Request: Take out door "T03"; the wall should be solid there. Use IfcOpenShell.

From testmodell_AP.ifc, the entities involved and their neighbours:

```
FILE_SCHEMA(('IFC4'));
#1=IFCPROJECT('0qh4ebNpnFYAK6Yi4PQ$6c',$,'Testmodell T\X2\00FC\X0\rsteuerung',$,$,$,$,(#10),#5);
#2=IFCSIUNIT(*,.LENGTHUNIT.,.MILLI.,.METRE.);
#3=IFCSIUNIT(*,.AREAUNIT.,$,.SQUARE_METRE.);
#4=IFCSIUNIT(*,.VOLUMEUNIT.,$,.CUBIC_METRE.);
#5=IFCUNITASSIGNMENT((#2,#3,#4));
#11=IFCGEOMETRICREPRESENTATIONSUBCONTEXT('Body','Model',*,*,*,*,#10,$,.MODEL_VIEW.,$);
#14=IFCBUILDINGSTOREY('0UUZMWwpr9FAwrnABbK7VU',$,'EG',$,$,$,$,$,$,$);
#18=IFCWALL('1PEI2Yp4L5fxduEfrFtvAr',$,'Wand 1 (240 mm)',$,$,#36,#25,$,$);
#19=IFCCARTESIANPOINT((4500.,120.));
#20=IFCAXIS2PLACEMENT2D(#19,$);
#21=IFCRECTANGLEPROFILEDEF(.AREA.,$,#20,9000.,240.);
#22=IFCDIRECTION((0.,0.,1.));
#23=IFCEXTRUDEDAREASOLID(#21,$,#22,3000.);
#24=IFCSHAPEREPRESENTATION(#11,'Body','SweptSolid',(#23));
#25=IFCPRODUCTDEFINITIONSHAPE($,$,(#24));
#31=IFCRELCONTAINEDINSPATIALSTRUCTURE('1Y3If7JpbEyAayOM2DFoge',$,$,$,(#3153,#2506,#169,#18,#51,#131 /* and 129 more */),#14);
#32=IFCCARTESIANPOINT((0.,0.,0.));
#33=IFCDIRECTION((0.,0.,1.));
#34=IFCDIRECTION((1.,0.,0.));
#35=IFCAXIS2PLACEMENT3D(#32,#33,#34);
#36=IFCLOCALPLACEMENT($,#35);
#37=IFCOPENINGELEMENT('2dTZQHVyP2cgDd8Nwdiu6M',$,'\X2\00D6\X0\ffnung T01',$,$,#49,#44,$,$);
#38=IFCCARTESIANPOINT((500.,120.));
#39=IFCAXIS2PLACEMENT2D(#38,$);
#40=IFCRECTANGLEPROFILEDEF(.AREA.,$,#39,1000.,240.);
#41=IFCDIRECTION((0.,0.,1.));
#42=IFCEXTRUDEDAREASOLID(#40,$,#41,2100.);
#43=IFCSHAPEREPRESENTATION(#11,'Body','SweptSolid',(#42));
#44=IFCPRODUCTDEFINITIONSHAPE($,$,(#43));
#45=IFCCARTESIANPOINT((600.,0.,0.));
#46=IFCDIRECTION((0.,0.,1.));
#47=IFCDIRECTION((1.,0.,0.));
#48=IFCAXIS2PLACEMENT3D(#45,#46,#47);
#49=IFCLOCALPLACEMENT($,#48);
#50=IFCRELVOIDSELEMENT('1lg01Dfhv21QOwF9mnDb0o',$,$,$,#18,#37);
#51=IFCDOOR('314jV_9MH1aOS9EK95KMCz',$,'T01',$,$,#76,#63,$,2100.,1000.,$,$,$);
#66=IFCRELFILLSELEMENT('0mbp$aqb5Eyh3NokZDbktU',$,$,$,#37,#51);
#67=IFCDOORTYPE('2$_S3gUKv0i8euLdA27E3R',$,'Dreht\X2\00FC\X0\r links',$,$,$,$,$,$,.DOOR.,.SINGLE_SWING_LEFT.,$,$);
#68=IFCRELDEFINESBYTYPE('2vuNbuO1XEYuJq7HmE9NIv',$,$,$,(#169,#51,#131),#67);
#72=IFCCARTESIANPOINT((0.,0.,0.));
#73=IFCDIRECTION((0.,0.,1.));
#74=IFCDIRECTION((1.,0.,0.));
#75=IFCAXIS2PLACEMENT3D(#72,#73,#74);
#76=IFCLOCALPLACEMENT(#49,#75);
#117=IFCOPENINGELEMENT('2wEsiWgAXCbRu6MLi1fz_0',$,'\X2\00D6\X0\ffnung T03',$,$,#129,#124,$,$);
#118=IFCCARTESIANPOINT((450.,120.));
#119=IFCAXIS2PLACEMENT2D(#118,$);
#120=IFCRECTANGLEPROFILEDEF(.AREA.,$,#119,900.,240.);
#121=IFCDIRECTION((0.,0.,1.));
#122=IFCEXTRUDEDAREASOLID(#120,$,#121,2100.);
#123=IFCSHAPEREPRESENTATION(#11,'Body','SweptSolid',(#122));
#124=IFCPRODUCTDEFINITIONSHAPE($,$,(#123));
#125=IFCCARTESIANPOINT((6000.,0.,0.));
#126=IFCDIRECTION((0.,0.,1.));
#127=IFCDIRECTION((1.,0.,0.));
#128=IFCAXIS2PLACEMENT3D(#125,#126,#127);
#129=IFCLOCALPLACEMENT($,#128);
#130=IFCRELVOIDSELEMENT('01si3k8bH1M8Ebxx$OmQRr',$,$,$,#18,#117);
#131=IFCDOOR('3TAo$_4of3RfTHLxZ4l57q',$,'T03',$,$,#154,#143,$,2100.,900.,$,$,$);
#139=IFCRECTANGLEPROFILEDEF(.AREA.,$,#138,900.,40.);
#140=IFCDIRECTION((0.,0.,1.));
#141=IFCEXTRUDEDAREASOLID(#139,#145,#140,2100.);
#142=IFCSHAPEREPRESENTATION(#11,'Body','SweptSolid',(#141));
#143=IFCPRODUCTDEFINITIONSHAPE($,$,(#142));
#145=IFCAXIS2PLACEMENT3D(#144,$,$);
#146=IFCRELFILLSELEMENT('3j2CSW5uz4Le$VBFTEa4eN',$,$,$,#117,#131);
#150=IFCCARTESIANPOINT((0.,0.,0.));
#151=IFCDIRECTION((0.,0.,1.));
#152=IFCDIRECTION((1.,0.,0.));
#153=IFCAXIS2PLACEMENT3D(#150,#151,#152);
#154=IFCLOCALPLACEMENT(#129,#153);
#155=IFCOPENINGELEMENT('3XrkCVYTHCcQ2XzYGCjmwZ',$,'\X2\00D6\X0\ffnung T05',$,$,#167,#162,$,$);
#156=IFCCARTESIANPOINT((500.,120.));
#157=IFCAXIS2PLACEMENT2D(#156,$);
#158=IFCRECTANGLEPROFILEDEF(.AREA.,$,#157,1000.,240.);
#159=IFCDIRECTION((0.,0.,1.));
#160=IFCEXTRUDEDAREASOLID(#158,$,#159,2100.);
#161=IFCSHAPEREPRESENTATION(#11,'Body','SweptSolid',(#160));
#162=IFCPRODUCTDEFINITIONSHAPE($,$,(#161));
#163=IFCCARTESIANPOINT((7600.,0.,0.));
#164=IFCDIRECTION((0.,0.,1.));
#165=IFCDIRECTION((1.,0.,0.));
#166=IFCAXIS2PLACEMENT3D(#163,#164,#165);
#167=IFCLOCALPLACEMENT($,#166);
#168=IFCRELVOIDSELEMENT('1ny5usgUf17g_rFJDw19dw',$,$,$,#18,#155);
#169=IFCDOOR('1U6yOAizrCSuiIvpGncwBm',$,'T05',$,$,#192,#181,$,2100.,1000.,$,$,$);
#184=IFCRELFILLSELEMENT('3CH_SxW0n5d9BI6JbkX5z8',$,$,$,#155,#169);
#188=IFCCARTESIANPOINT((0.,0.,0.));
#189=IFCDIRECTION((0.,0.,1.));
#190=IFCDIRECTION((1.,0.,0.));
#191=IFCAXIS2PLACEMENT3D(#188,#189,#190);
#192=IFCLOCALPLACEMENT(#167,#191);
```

```python
import ifcopenshell
import ifcopenshell.api.feature
import ifcopenshell.api.root
import ifcopenshell.geom
import ifcopenshell.util.shape

model = ifcopenshell.open("testmodell_AP.ifc")
settings = ifcopenshell.geom.settings()


def volume(element):
    """Net volume in cubic metres, openings subtracted."""
    shape = ifcopenshell.geom.create_shape(settings, element)
    return ifcopenshell.util.shape.get_volume(shape.geometry)


door = model.by_guid("3TAo$_4of3RfTHLxZ4l57q")
opening = door.FillsVoids[0].RelatingOpeningElement
wall = opening.VoidsElements[0].RelatingBuildingElement
before = volume(wall)

ifcopenshell.api.root.remove_product(model, product=door)
ifcopenshell.api.feature.remove_feature(model, feature=opening)

after = volume(wall)

print(f"wall volume {before:.3f} -> {after:.3f} m3")

model.write("testmodell_AP_updated.ifc")
```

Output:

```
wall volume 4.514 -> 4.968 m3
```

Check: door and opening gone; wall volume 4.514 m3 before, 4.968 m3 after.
